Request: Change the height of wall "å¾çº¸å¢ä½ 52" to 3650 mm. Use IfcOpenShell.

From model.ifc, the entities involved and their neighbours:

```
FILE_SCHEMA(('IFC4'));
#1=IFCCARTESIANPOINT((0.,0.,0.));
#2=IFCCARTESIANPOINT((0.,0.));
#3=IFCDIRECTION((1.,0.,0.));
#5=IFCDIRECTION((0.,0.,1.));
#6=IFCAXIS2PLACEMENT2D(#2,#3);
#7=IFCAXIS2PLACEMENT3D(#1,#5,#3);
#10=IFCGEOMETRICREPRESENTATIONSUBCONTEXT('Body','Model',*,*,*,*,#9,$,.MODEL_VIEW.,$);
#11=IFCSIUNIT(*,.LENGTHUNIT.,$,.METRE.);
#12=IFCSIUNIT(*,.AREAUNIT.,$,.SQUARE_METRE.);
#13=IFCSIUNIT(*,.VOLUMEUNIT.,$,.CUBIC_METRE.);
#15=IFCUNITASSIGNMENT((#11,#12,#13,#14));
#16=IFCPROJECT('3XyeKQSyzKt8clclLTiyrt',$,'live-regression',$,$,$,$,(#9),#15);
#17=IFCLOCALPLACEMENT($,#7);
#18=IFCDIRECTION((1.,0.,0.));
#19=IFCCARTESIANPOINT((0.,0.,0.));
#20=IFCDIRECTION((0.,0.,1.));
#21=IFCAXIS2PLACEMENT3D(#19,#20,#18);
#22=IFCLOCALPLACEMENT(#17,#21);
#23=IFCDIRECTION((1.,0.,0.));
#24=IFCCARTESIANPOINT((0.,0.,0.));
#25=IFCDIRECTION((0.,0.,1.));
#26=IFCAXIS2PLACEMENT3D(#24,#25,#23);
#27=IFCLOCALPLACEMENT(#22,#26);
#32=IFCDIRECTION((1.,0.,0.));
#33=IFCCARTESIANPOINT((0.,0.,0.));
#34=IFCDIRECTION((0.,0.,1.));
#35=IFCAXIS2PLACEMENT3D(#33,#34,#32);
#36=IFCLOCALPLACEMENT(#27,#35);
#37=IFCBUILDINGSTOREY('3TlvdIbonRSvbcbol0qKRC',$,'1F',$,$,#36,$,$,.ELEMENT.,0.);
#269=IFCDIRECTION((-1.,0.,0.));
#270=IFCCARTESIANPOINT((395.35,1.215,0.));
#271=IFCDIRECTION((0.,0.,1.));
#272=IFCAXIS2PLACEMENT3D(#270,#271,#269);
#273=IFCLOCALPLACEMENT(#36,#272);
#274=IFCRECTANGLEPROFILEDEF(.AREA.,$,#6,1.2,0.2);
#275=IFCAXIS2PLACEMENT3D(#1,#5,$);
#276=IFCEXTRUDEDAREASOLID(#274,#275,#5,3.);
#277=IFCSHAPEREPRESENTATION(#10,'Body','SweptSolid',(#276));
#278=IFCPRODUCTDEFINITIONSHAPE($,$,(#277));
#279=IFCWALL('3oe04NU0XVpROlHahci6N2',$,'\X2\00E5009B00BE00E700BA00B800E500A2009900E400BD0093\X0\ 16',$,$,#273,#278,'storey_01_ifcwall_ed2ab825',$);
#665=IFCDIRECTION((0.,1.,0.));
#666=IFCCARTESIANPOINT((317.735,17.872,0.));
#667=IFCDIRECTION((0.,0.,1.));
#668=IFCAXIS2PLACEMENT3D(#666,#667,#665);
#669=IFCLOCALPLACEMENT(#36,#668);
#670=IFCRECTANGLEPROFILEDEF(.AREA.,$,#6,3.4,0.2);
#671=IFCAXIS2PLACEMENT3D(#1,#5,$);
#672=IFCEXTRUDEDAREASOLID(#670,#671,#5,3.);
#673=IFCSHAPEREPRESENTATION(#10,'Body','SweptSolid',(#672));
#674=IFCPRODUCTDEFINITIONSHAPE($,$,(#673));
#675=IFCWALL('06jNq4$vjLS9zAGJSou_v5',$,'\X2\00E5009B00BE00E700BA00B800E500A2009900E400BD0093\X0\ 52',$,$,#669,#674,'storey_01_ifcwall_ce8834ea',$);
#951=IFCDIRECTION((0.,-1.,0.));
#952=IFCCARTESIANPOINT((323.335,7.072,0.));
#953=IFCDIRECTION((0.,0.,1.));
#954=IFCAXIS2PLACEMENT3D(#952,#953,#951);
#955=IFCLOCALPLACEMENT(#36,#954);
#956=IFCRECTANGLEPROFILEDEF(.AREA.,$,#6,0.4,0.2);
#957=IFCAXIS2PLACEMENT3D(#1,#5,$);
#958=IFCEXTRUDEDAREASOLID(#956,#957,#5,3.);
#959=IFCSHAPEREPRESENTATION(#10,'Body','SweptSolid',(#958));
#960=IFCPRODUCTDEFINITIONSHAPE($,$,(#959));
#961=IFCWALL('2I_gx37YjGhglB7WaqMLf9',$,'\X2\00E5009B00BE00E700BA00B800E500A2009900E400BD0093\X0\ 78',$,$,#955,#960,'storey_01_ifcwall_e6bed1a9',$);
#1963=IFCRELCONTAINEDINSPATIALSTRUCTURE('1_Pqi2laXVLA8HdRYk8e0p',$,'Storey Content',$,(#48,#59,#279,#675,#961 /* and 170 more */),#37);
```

```python
import ifcopenshell
import ifcopenshell.geom
import ifcopenshell.util.representation
import ifcopenshell.util.shape
import ifcopenshell.util.unit

model = ifcopenshell.open("model.ifc")
unit_scale = ifcopenshell.util.unit.calculate_unit_scale(model)
settings = ifcopenshell.geom.settings()


def volume(element):
    """Net volume in cubic metres, openings subtracted."""
    shape = ifcopenshell.geom.create_shape(settings, element)
    return ifcopenshell.util.shape.get_volume(shape.geometry)


wall = model.by_id(675)
before = volume(wall)

body = ifcopenshell.util.representation.get_representation(wall, "Model", "Body")
solid = body.Items[0]
old_height = solid.Depth
solid.Depth = 3.65 / unit_scale
after = volume(wall)

print(f"height {old_height:g} -> {solid.Depth:g}, volume {before:.3f} -> {after:.3f} m3")

model.write("model_v2.ifc")
```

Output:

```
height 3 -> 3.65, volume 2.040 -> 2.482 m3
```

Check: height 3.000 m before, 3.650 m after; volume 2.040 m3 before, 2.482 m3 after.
